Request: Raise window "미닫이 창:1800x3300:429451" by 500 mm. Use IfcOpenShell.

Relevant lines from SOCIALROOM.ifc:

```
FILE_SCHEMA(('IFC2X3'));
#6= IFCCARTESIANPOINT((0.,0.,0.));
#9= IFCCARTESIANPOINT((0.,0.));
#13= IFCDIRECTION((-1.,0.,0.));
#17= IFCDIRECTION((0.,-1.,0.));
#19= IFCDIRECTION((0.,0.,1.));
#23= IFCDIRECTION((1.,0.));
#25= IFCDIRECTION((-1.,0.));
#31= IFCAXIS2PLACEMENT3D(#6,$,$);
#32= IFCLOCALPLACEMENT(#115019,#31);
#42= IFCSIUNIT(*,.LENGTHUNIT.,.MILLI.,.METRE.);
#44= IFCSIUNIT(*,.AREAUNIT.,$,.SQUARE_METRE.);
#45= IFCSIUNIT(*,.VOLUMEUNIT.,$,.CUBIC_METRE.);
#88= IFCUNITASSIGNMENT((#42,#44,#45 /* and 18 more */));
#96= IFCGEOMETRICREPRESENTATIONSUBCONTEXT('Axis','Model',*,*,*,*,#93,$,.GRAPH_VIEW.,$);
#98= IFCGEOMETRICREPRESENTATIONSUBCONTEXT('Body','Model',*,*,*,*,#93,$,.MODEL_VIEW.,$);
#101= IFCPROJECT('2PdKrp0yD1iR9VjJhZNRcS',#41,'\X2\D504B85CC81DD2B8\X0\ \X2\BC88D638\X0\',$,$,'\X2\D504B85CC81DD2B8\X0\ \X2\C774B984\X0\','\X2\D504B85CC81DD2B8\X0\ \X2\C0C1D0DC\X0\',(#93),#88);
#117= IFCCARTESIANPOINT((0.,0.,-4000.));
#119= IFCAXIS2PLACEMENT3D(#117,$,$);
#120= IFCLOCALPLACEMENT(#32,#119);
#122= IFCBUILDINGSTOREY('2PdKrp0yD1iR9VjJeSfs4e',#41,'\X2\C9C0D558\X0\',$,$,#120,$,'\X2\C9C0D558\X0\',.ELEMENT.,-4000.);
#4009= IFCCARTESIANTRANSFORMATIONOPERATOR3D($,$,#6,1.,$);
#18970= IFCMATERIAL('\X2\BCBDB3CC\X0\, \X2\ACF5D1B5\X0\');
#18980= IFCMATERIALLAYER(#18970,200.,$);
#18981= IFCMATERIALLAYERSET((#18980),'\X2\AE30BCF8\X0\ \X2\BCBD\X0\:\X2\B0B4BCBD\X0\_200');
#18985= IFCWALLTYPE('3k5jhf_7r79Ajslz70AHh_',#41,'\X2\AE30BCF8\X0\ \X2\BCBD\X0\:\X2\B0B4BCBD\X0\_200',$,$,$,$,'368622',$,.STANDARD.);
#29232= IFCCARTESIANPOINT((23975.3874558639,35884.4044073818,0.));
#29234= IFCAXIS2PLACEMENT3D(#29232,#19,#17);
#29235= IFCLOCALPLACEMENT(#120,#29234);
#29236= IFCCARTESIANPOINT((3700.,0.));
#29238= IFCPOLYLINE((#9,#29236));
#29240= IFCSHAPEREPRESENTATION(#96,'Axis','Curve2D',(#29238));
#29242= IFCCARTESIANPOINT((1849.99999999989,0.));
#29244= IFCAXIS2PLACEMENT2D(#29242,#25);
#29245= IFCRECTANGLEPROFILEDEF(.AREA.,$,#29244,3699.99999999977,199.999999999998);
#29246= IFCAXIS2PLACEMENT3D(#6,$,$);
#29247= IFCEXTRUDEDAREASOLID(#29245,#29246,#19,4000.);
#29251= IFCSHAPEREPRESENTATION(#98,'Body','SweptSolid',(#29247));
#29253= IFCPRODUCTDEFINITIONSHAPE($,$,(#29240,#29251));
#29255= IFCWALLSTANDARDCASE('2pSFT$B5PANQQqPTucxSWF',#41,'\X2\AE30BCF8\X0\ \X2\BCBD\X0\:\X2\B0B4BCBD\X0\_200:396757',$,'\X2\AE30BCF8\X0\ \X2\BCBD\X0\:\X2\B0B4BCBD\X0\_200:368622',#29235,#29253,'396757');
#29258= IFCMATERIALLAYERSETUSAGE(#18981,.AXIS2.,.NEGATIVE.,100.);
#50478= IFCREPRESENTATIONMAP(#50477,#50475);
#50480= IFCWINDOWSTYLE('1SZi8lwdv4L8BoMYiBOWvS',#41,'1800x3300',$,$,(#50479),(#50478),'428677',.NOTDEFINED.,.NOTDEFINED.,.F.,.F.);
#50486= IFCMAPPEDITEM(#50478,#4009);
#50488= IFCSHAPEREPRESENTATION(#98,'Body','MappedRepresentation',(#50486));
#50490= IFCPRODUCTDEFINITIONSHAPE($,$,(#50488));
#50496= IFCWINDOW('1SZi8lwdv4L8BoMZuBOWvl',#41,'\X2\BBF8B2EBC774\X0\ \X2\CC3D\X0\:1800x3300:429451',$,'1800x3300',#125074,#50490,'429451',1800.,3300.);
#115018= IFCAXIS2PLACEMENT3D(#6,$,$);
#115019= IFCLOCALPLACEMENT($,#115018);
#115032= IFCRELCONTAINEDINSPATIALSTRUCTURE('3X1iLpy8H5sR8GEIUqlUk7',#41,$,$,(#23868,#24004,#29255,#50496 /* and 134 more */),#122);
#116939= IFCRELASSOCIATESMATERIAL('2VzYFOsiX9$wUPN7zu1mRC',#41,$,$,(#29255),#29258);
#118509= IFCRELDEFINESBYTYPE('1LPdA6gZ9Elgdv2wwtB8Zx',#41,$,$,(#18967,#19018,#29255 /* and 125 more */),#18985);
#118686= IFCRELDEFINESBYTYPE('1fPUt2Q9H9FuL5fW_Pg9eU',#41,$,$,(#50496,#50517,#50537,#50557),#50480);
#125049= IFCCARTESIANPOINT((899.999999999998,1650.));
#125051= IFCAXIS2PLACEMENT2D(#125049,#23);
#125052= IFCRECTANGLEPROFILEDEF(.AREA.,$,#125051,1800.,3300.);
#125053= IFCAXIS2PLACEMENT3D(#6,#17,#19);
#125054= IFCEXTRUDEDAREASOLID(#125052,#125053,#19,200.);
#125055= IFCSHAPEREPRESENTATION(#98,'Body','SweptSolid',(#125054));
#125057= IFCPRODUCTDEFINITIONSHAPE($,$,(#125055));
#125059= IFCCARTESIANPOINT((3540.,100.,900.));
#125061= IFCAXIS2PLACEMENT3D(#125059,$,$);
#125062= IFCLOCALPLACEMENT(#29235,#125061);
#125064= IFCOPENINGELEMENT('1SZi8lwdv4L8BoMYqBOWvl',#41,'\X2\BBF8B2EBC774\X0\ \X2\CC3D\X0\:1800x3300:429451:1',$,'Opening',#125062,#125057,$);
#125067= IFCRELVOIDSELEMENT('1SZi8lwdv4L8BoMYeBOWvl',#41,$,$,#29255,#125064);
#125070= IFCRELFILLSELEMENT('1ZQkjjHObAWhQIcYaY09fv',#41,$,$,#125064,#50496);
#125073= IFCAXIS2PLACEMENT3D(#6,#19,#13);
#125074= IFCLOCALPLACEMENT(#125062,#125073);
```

```python
import numpy as np
import ifcopenshell
import ifcopenshell.api.geometry
import ifcopenshell.util.placement
import ifcopenshell.util.unit

model = ifcopenshell.open("SOCIALROOM.ifc")
unit_scale = ifcopenshell.util.unit.calculate_unit_scale(model)

window = model.by_guid("1SZi8lwdv4L8BoMZuBOWvl")
opening = window.FillsVoids[0].RelatingOpeningElement
dz = 500.0

shift = np.array([0.0, 0.0, dz])
# The window is placed relative to its opening, so it follows when the opening moves.
matrix = ifcopenshell.util.placement.get_local_placement(opening.ObjectPlacement)
matrix[:3, 3] += shift
ifcopenshell.api.geometry.edit_object_placement(
    model, product=opening, matrix=matrix, is_si=False, should_transform_children=True
)

print(f"moved by {dz * unit_scale:+.3f} m")

model.write("SOCIALROOM_edited.ifc")
```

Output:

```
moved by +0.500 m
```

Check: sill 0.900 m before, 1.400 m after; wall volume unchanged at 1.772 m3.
